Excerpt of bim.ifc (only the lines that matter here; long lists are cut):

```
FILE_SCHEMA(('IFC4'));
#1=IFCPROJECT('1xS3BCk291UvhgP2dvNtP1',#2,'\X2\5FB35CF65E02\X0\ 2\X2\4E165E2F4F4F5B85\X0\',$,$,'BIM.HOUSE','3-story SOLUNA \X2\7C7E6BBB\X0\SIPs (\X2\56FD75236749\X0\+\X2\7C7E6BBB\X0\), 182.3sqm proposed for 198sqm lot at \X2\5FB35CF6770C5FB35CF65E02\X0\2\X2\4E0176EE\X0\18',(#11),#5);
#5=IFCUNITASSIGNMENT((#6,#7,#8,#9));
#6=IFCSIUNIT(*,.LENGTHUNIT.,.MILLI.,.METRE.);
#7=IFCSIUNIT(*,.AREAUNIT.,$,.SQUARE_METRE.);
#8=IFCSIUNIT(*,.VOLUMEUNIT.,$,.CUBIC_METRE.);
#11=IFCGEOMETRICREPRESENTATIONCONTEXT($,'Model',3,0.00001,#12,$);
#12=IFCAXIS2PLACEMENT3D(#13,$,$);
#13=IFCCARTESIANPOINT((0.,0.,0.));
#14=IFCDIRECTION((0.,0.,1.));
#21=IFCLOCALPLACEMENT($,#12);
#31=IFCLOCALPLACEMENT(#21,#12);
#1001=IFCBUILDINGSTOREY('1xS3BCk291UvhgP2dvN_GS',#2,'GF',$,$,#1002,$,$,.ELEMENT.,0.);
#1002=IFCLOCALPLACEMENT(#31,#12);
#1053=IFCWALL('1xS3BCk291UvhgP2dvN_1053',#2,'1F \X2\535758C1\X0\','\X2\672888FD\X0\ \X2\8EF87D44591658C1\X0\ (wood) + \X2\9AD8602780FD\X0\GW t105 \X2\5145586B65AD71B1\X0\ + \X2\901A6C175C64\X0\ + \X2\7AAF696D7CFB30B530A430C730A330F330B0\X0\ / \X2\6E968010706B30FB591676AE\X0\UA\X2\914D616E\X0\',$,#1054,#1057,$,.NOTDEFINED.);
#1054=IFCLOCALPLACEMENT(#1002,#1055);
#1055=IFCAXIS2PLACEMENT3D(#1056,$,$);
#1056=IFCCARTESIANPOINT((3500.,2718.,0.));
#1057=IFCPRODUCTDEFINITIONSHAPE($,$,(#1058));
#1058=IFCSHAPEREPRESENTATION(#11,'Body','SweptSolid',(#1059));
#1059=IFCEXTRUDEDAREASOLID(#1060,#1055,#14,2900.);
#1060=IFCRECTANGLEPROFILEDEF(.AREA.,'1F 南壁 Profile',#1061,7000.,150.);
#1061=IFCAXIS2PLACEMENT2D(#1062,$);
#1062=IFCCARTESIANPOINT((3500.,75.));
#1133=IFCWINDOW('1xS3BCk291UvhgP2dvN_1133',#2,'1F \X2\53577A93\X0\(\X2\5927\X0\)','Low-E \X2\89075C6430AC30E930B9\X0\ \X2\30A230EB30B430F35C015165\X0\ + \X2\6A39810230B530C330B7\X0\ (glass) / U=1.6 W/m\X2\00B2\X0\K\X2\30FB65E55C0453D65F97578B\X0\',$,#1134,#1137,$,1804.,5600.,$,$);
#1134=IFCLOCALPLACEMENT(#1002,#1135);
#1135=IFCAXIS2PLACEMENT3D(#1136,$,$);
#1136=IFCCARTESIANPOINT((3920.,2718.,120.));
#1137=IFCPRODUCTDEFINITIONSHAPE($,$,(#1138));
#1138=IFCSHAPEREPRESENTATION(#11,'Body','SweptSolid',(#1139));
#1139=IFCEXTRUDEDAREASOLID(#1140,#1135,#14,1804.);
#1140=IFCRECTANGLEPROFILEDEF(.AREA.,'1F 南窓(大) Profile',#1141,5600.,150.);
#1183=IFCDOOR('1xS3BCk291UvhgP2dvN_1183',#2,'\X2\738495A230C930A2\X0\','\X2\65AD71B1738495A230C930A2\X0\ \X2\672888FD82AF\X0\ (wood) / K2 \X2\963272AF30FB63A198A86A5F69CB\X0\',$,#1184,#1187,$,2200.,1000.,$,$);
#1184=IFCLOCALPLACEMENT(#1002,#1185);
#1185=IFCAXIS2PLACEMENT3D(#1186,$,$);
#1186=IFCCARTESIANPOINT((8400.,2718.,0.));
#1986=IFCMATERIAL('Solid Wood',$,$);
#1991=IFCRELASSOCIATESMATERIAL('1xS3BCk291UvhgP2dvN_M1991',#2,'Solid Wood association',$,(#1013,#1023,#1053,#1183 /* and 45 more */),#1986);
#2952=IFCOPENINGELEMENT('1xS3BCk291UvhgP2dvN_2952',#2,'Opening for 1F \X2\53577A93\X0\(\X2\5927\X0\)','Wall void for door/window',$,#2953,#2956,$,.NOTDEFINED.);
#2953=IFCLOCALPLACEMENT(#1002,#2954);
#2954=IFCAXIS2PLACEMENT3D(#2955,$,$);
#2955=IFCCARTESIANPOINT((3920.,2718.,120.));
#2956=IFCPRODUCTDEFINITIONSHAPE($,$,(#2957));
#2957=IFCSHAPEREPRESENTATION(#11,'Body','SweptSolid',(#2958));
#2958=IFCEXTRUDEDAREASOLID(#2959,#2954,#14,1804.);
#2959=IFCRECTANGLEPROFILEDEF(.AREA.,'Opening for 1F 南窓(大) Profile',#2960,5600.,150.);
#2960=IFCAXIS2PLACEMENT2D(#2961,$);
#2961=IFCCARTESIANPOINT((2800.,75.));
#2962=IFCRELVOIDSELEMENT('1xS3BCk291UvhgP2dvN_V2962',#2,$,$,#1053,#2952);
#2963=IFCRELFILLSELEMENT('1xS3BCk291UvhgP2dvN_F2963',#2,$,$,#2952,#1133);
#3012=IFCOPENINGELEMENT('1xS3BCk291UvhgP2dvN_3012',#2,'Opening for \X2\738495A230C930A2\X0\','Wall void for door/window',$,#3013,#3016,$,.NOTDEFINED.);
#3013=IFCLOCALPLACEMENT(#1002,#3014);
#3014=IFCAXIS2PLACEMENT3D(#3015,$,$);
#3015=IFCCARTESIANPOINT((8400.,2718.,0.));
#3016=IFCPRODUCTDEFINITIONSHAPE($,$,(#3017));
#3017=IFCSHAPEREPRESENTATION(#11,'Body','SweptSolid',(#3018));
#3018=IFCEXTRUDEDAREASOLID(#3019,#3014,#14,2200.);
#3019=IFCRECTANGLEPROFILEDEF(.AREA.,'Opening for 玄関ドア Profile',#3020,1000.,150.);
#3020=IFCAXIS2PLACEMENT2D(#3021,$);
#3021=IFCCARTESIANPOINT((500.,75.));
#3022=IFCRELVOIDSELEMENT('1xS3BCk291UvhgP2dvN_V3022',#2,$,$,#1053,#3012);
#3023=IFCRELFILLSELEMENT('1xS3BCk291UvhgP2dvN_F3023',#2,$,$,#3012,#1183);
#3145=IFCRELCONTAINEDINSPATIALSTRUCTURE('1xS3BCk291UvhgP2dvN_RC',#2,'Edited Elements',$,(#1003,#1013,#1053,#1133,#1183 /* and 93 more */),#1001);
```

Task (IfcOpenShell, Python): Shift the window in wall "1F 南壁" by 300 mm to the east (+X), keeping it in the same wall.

```python
import ifcopenshell
import ifcopenshell.api.geometry
import ifcopenshell.util.placement
import ifcopenshell.util.unit

model = ifcopenshell.open("bim.ifc")
unit_scale = ifcopenshell.util.unit.calculate_unit_scale(model)

window = model.by_guid("1xS3BCk291UvhgP2dvN_1133")
opening = window.FillsVoids[0].RelatingOpeningElement
wall = opening.VoidsElements[0].RelatingBuildingElement

wall_matrix = ifcopenshell.util.placement.get_local_placement(wall.ObjectPlacement)
shift = wall_matrix[:3, 0] * 0.3 / unit_scale
before = ifcopenshell.util.placement.get_local_placement(window.ObjectPlacement)[:3, 3].copy()

# The window is not placed relative to its opening, so move both.
for product in (opening, window):
    matrix = ifcopenshell.util.placement.get_local_placement(product.ObjectPlacement)
    matrix[:3, 3] += shift
    ifcopenshell.api.geometry.edit_object_placement(model, product=product, matrix=matrix, is_si=False)

after = ifcopenshell.util.placement.get_local_placement(window.ObjectPlacement)[:3, 3]
print("window moved by", (after - before).round(3) + 0.0)

model.write("bim_rev.ifc")
```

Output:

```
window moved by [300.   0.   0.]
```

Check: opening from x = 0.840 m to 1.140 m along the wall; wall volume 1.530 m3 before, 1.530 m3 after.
